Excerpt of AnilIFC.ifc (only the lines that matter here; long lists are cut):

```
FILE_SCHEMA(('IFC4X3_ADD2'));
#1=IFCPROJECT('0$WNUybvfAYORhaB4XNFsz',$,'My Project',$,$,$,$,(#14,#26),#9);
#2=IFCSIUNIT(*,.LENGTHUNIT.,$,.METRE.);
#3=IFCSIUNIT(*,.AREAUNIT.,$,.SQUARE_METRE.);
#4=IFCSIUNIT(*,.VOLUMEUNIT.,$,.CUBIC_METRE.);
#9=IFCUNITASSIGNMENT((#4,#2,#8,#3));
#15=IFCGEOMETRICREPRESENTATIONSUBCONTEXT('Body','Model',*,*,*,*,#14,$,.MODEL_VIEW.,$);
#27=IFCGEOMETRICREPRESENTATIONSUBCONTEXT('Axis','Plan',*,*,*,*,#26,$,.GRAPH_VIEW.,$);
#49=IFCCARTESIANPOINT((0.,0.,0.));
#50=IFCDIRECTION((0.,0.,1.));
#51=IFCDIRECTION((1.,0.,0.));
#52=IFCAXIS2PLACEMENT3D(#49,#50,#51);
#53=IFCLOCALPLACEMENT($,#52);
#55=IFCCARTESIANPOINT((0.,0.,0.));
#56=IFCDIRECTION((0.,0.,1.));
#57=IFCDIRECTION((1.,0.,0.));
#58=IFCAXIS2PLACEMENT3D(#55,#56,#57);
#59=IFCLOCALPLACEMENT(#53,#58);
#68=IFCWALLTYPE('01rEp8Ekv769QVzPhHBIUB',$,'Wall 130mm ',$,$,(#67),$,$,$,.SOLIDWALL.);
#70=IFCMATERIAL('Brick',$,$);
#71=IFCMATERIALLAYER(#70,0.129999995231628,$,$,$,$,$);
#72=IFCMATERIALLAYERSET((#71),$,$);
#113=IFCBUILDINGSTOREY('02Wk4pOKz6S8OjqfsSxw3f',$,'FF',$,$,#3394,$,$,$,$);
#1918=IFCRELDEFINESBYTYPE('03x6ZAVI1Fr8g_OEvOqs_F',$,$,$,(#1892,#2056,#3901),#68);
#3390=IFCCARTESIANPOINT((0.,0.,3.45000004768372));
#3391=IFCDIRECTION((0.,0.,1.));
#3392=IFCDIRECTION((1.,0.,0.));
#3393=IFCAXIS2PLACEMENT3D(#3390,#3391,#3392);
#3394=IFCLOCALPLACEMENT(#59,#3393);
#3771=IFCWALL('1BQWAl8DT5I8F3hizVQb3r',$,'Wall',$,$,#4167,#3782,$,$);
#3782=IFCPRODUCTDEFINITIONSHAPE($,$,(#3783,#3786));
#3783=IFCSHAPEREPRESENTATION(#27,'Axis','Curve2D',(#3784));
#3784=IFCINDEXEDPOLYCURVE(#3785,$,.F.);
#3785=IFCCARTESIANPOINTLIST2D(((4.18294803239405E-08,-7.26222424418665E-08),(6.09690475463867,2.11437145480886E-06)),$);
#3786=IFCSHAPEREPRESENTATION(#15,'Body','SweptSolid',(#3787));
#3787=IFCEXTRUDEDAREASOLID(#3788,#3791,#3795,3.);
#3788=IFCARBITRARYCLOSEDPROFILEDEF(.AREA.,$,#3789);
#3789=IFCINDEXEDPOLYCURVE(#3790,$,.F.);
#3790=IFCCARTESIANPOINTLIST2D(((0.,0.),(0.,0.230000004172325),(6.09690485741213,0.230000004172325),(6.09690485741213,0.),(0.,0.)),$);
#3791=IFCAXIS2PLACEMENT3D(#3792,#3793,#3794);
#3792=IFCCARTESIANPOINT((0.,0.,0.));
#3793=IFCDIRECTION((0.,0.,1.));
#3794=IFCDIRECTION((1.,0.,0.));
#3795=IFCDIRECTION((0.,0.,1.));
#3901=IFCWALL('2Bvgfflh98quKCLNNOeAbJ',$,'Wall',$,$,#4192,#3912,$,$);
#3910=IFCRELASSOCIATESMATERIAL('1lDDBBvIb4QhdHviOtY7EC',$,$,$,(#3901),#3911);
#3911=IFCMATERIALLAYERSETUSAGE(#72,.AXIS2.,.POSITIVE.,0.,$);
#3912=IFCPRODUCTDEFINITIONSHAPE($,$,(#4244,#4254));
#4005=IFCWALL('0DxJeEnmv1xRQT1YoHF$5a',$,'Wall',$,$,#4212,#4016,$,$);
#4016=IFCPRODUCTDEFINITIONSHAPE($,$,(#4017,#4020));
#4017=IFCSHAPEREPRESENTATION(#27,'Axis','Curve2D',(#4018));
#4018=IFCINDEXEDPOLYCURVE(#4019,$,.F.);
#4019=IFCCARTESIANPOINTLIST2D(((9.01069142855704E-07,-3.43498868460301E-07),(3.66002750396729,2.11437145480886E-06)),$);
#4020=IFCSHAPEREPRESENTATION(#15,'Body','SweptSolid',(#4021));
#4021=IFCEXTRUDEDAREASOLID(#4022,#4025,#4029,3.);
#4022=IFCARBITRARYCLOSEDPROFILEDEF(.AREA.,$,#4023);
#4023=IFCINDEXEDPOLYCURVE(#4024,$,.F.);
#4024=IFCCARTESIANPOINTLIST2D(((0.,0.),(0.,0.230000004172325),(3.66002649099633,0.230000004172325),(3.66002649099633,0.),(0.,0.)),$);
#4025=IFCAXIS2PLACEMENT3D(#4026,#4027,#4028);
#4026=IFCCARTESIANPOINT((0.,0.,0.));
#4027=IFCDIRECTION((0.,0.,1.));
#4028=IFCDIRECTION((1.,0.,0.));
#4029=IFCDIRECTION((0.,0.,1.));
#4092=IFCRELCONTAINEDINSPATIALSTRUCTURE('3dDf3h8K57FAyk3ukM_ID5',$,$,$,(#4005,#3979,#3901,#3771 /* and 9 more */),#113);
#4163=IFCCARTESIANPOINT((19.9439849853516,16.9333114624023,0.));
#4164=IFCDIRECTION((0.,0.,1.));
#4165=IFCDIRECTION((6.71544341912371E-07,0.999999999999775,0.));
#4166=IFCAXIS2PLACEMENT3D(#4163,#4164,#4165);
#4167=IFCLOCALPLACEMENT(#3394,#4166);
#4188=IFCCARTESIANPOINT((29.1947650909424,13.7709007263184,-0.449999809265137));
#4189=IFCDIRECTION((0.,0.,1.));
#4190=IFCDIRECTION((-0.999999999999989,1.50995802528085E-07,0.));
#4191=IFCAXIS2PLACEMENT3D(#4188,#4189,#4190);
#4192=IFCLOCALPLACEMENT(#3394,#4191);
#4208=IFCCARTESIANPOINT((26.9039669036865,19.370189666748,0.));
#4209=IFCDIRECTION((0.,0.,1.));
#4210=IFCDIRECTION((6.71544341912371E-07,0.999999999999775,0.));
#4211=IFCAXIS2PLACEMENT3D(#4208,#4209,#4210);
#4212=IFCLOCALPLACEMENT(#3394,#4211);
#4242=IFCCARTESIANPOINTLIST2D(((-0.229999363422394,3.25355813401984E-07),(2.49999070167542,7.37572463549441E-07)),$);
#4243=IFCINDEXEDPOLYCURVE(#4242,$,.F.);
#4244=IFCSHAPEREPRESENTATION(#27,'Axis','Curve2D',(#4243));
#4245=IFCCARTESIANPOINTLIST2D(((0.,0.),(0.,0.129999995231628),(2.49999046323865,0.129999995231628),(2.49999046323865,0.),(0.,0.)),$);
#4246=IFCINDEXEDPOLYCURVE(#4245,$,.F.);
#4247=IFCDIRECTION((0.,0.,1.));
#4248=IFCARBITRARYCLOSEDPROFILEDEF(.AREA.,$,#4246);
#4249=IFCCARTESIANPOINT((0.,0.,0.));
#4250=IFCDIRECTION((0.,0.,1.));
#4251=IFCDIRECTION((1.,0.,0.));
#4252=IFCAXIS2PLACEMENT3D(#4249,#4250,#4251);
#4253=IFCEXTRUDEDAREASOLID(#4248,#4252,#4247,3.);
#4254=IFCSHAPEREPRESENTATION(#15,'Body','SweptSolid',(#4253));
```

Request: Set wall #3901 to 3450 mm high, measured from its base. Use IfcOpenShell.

```python
import ifcopenshell
import ifcopenshell.geom
import ifcopenshell.util.representation
import ifcopenshell.util.shape
import ifcopenshell.util.unit

model = ifcopenshell.open("AnilIFC.ifc")
unit_scale = ifcopenshell.util.unit.calculate_unit_scale(model)
settings = ifcopenshell.geom.settings()


def volume(element):
    """Net volume in cubic metres, openings subtracted."""
    shape = ifcopenshell.geom.create_shape(settings, element)
    return ifcopenshell.util.shape.get_volume(shape.geometry)


wall = model.by_guid("2Bvgfflh98quKCLNNOeAbJ")
before = volume(wall)

body = ifcopenshell.util.representation.get_representation(wall, "Model", "Body")
solid = body.Items[0]
old_height = solid.Depth
solid.Depth = 3.45 / unit_scale
after = volume(wall)

print(f"height {old_height:g} -> {solid.Depth:g}, volume {before:.3f} -> {after:.3f} m3")

model.write("AnilIFC_rev.ifc")
```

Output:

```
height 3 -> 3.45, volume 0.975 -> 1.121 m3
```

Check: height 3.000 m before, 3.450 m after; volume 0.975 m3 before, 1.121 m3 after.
